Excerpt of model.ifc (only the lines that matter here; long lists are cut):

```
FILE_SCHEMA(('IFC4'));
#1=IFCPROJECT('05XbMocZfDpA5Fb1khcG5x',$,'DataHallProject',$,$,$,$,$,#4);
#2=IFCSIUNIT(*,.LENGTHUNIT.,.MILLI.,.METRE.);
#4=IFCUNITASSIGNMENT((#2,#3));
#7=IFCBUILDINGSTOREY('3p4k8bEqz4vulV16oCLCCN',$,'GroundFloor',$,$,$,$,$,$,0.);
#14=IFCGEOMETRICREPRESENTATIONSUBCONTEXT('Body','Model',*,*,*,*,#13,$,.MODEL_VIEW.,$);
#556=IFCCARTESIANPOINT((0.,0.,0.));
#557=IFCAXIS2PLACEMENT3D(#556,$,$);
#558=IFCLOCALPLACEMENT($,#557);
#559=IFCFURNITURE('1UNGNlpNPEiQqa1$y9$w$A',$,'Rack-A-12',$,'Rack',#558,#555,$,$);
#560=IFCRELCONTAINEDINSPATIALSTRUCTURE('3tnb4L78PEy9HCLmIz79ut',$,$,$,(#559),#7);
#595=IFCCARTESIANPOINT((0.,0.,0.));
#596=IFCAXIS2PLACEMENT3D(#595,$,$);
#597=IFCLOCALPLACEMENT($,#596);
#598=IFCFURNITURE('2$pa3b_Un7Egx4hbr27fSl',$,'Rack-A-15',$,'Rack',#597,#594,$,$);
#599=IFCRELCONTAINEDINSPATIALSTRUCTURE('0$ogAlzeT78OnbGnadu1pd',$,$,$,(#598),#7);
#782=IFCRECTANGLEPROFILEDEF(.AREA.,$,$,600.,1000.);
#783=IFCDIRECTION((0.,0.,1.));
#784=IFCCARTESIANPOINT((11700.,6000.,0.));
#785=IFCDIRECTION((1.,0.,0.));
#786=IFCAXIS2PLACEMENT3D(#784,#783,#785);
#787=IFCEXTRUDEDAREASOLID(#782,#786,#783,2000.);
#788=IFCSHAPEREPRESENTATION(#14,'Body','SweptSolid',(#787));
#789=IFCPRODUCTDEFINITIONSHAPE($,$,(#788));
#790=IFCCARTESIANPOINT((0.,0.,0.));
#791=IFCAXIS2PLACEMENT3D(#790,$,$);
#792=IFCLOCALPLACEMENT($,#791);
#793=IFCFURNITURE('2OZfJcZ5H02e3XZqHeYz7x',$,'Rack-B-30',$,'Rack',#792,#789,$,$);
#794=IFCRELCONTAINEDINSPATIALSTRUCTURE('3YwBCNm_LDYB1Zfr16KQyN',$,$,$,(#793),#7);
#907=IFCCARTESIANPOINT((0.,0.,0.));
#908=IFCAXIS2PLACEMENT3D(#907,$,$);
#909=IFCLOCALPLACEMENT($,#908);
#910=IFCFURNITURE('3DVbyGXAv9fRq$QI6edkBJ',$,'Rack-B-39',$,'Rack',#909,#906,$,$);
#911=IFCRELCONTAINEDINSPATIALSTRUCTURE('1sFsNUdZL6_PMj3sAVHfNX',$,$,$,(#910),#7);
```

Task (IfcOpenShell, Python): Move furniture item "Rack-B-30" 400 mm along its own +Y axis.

```python
import ifcopenshell
import ifcopenshell.api.geometry
import ifcopenshell.util.placement

model = ifcopenshell.open("model.ifc")

item = model.by_id(793)
matrix = ifcopenshell.util.placement.get_local_placement(item.ObjectPlacement)
matrix[:3, 3] += matrix[:3, 1] * 400.0
ifcopenshell.api.geometry.edit_object_placement(model, product=item, matrix=matrix, is_si=False)

print(ifcopenshell.util.placement.get_local_placement(item.ObjectPlacement).round(3) + 0.0)

model.write("model_v2.ifc")
```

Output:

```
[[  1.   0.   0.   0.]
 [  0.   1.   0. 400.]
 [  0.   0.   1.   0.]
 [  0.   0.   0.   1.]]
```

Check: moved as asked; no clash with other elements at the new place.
